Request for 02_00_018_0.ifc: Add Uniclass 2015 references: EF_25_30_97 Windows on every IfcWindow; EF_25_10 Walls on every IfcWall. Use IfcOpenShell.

First a look at what the model holds.

```python
import ifcopenshell

model = ifcopenshell.open("02_00_018_0.ifc")
print(model.schema)
print("classifications:", [c.Name for c in model.by_type("IfcClassification")])
for ifc_class in ("IfcDoor", "IfcRoof", "IfcStair", "IfcWall", "IfcWindow"):
    print(ifc_class, len(model.by_type(ifc_class)))
```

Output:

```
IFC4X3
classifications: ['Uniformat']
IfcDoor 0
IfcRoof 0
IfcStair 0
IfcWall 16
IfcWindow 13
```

```python
import ifcopenshell
import ifcopenshell.api.classification

model = ifcopenshell.open("02_00_018_0.ifc")

system = ifcopenshell.api.classification.add_classification(model, classification="Uniclass 2015")

codes = {
    "IfcWindow": ("EF_25_30_97", "Windows"),
    "IfcWall": ("EF_25_10", "Walls"),
}
for ifc_class, (code, name) in codes.items():
    products = model.by_type(ifc_class)
    ifcopenshell.api.classification.add_reference(
        model, products=products, classification=system, identification=code, name=name
    )
    print(code, len(products))

model.write("02_00_018_0_updated.ifc")
```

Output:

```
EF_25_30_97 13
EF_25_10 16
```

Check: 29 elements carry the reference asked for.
